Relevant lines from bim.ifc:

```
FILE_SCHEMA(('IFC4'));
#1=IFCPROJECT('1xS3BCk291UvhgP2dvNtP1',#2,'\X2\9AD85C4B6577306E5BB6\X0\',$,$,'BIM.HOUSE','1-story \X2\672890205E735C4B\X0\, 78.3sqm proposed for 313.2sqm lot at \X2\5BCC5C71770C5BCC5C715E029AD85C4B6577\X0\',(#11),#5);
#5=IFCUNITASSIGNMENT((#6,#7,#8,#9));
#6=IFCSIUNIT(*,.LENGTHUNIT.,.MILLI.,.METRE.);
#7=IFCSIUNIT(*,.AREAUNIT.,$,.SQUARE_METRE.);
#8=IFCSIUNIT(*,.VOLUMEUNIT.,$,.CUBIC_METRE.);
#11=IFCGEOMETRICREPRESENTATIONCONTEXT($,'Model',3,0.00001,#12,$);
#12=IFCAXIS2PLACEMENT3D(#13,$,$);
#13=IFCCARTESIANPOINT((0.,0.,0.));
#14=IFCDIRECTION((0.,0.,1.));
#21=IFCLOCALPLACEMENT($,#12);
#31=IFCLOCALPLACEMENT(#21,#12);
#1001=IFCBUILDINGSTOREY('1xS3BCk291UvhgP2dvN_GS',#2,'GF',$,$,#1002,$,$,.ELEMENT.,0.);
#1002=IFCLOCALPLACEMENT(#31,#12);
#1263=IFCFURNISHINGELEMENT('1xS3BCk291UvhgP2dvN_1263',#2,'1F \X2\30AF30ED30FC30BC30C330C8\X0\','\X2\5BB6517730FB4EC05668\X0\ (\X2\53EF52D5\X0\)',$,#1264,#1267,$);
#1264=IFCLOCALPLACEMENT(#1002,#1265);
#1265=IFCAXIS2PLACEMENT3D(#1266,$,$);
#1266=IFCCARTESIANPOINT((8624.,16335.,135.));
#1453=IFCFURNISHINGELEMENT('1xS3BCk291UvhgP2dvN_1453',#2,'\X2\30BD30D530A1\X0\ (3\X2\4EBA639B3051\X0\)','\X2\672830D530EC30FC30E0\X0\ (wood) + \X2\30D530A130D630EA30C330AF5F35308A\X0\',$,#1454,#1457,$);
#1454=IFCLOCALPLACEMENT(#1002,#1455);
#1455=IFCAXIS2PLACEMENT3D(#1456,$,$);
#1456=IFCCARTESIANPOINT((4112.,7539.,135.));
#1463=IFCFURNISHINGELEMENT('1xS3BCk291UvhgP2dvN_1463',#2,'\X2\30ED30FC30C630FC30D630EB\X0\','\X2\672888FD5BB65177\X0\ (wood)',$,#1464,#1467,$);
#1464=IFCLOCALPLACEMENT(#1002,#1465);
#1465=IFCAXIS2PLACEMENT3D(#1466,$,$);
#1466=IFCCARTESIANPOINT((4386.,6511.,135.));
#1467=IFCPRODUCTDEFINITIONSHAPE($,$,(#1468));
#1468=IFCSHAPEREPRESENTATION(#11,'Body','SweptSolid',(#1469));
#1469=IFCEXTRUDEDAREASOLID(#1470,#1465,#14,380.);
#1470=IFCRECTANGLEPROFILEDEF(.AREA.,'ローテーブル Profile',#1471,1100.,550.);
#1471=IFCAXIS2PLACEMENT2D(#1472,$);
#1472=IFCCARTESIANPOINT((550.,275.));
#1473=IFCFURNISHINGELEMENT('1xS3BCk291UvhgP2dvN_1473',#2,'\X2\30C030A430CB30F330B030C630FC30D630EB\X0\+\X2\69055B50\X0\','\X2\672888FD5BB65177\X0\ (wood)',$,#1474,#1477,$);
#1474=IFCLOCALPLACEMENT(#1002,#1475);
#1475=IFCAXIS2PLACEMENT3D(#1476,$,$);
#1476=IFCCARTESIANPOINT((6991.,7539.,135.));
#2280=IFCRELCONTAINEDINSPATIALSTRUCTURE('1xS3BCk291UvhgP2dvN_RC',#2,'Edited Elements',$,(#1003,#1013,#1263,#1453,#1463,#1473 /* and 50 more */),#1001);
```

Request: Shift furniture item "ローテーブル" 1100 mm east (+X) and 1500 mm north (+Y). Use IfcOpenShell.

```python
import ifcopenshell
import ifcopenshell.api.geometry
import ifcopenshell.util.placement

model = ifcopenshell.open("bim.ifc")

item = model.by_guid("1xS3BCk291UvhgP2dvN_1463")
matrix = ifcopenshell.util.placement.get_local_placement(item.ObjectPlacement)
matrix[0, 3] += 1100.0
matrix[1, 3] += 1500.0
ifcopenshell.api.geometry.edit_object_placement(model, product=item, matrix=matrix, is_si=False)

print(ifcopenshell.util.placement.get_local_placement(item.ObjectPlacement).round(3) + 0.0)

model.write("bim-out.ifc")
```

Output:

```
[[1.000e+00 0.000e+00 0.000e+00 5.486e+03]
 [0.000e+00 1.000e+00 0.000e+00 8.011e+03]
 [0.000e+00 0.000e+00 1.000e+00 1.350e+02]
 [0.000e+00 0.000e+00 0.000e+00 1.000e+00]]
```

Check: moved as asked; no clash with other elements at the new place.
